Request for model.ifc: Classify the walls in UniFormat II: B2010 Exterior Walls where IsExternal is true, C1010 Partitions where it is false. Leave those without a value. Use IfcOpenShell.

First a look at what the model holds.

```python
import ifcopenshell
import ifcopenshell.util.element

model = ifcopenshell.open("model.ifc")
print(model.schema)
print("classifications:", [c.Name for c in model.by_type("IfcClassification")])
values = [ifcopenshell.util.element.get_pset(e, "Pset_WallCommon", "IsExternal") for e in model.by_type("IfcWall")]
for value in (True, False, None):
    print("IsExternal", value, values.count(value))
```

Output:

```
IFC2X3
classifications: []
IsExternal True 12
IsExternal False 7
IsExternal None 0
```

```python
import ifcopenshell
import ifcopenshell.api.classification
import ifcopenshell.util.element

model = ifcopenshell.open("model.ifc")

# IFC2X3 requires Source and Edition and has no link from the project to the system.
system = model.create_entity("IfcClassification", Source="ASTM", Edition="E1557", Name="UniFormat II")

walls = model.by_type("IfcWall")
external = {e: ifcopenshell.util.element.get_pset(e, "Pset_WallCommon", "IsExternal") for e in walls}
for flag, code, name in ((True, "B2010", "Exterior Walls"), (False, "C1010", "Partitions")):
    products = [e for e in walls if external[e] is flag]
    ifcopenshell.api.classification.add_reference(
        model, products=products, classification=system, identification=code, name=name
    )
    print(code, len(products))

model.write("model_updated.ifc")
```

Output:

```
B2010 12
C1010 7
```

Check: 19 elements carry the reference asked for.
